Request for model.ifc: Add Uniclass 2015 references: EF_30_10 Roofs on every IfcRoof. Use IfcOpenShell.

First a look at what the model holds.

```python
import ifcopenshell

model = ifcopenshell.open("model.ifc")
print(model.schema)
print("classifications:", [c.Name for c in model.by_type("IfcClassification")])
for ifc_class in ("IfcDoor", "IfcRoof", "IfcStair", "IfcWall", "IfcWindow"):
    print(ifc_class, len(model.by_type(ifc_class)))
```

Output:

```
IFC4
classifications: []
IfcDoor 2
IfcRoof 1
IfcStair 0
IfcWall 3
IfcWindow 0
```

```python
import ifcopenshell
import ifcopenshell.api.classification

model = ifcopenshell.open("model.ifc")

system = ifcopenshell.api.classification.add_classification(model, classification="Uniclass 2015")

codes = {
    "IfcRoof": ("EF_30_10", "Roofs"),
}
for ifc_class, (code, name) in codes.items():
    products = model.by_type(ifc_class)
    ifcopenshell.api.classification.add_reference(
        model, products=products, classification=system, identification=code, name=name
    )
    print(code, len(products))

model.write("model_updated.ifc")
```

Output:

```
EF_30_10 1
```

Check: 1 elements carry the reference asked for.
